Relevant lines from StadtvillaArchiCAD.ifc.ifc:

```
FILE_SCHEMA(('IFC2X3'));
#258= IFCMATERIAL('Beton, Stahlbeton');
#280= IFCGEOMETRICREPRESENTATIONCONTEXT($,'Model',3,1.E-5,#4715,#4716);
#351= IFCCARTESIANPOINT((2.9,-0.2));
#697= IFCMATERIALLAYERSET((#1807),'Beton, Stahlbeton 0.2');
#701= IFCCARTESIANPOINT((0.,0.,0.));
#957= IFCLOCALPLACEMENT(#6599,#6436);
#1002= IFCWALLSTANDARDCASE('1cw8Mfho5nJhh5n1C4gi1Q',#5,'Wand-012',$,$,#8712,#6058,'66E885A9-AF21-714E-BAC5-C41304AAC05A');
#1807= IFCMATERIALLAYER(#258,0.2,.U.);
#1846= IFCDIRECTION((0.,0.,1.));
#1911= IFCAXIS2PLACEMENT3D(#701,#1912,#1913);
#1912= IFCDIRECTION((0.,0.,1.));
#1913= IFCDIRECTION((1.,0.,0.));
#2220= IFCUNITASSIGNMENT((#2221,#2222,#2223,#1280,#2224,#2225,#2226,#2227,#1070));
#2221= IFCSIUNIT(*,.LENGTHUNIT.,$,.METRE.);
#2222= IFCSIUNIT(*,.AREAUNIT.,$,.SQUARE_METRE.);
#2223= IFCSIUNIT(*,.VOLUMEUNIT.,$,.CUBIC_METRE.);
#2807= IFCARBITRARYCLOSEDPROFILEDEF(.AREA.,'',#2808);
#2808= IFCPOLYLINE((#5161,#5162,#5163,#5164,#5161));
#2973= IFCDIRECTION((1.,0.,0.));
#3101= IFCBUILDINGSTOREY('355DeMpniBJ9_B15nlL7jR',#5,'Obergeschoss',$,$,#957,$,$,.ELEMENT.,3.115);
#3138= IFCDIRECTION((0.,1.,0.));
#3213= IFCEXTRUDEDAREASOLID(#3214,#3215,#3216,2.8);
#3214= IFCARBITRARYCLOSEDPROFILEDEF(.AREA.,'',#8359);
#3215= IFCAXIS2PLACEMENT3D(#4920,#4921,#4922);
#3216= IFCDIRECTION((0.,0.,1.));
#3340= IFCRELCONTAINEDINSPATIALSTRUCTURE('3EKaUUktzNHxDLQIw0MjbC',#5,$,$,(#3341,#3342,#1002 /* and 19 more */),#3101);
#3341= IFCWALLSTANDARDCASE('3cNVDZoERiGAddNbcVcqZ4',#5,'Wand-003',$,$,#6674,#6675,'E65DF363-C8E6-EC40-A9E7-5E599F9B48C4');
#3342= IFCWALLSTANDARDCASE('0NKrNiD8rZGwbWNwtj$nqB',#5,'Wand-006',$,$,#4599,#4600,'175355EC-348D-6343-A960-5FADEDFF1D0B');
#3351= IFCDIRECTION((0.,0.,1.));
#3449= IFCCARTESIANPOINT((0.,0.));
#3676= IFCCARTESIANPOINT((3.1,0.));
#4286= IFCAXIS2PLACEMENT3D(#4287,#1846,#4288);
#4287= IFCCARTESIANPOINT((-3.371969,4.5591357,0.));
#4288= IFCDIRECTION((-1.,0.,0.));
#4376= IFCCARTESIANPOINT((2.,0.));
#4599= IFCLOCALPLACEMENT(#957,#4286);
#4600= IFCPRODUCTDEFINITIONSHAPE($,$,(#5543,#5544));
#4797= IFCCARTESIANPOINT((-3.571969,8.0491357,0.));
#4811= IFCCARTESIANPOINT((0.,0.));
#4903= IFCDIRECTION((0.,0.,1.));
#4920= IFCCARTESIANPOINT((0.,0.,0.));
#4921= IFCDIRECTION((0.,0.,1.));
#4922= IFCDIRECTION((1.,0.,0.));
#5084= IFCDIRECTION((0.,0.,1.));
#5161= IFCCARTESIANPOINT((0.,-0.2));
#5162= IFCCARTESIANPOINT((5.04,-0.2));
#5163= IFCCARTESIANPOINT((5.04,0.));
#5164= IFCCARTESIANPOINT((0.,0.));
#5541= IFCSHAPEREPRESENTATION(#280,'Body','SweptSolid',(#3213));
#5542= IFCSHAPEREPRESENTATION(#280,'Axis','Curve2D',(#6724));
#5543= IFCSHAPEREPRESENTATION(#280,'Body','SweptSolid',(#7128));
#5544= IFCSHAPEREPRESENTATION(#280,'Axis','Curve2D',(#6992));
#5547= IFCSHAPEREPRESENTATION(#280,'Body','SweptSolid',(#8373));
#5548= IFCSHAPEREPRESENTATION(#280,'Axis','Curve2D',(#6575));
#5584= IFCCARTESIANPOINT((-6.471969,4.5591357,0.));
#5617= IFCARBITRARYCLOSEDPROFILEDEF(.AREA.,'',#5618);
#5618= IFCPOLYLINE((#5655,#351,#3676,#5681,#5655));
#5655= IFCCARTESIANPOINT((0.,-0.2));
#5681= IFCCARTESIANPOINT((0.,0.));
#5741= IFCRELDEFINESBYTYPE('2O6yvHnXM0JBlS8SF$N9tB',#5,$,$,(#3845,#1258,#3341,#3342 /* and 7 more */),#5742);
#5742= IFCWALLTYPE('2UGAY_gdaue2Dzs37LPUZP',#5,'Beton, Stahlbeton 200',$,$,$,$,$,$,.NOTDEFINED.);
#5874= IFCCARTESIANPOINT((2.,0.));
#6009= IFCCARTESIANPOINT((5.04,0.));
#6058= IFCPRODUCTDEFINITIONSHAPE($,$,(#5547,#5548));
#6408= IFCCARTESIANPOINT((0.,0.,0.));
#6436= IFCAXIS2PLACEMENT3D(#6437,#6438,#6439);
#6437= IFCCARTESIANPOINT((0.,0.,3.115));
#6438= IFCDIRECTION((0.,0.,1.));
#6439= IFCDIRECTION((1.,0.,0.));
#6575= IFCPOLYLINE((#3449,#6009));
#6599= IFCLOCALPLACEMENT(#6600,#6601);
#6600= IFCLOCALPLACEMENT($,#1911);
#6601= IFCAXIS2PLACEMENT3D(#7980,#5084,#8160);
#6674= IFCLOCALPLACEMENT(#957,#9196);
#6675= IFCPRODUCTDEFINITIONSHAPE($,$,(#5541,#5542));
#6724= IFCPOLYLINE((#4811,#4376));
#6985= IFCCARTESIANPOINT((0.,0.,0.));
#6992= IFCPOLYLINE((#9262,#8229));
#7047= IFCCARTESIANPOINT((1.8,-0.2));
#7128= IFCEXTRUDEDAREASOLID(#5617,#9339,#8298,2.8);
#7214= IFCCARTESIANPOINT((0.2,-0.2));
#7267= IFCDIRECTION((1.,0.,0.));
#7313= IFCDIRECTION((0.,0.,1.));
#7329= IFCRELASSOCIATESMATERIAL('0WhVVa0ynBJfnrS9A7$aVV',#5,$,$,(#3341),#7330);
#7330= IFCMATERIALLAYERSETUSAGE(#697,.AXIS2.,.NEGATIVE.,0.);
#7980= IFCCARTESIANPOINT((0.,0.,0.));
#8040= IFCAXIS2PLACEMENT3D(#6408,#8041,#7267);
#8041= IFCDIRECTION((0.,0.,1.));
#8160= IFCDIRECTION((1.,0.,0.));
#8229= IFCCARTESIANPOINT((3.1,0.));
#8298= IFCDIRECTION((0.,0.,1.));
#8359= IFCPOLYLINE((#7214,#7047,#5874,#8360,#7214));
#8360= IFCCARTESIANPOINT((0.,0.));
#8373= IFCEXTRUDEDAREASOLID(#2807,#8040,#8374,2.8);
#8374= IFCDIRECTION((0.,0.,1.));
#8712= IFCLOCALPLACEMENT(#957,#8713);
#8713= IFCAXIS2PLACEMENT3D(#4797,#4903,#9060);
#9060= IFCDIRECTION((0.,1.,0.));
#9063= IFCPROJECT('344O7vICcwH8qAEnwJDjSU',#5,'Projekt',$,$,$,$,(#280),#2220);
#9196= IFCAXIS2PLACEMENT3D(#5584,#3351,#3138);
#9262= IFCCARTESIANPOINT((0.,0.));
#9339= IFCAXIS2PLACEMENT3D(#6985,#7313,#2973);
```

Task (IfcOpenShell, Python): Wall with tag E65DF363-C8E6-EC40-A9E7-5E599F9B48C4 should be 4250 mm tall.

```python
import ifcopenshell
import ifcopenshell.geom
import ifcopenshell.util.shape

model = ifcopenshell.open("StadtvillaArchiCAD.ifc.ifc")
settings = ifcopenshell.geom.settings()


def volume(element):
    """Net volume in cubic metres, openings subtracted."""
    shape = ifcopenshell.geom.create_shape(settings, element)
    return ifcopenshell.util.shape.get_volume(shape.geometry)


wall = model.by_id(3341)
before = volume(wall)

body = next(r for r in wall.Representation.Representations if r.RepresentationIdentifier == "Body")
solid = body.Items[0]
old_height = solid.Depth
solid.Depth = 4.25
after = volume(wall)

print(f"height {old_height:g} -> {solid.Depth:g}, volume {before:.3f} -> {after:.3f} m3")

model.write("StadtvillaArchiCAD.ifc_updated.ifc")
```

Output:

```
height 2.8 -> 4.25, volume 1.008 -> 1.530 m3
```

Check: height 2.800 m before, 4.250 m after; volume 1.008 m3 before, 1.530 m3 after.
